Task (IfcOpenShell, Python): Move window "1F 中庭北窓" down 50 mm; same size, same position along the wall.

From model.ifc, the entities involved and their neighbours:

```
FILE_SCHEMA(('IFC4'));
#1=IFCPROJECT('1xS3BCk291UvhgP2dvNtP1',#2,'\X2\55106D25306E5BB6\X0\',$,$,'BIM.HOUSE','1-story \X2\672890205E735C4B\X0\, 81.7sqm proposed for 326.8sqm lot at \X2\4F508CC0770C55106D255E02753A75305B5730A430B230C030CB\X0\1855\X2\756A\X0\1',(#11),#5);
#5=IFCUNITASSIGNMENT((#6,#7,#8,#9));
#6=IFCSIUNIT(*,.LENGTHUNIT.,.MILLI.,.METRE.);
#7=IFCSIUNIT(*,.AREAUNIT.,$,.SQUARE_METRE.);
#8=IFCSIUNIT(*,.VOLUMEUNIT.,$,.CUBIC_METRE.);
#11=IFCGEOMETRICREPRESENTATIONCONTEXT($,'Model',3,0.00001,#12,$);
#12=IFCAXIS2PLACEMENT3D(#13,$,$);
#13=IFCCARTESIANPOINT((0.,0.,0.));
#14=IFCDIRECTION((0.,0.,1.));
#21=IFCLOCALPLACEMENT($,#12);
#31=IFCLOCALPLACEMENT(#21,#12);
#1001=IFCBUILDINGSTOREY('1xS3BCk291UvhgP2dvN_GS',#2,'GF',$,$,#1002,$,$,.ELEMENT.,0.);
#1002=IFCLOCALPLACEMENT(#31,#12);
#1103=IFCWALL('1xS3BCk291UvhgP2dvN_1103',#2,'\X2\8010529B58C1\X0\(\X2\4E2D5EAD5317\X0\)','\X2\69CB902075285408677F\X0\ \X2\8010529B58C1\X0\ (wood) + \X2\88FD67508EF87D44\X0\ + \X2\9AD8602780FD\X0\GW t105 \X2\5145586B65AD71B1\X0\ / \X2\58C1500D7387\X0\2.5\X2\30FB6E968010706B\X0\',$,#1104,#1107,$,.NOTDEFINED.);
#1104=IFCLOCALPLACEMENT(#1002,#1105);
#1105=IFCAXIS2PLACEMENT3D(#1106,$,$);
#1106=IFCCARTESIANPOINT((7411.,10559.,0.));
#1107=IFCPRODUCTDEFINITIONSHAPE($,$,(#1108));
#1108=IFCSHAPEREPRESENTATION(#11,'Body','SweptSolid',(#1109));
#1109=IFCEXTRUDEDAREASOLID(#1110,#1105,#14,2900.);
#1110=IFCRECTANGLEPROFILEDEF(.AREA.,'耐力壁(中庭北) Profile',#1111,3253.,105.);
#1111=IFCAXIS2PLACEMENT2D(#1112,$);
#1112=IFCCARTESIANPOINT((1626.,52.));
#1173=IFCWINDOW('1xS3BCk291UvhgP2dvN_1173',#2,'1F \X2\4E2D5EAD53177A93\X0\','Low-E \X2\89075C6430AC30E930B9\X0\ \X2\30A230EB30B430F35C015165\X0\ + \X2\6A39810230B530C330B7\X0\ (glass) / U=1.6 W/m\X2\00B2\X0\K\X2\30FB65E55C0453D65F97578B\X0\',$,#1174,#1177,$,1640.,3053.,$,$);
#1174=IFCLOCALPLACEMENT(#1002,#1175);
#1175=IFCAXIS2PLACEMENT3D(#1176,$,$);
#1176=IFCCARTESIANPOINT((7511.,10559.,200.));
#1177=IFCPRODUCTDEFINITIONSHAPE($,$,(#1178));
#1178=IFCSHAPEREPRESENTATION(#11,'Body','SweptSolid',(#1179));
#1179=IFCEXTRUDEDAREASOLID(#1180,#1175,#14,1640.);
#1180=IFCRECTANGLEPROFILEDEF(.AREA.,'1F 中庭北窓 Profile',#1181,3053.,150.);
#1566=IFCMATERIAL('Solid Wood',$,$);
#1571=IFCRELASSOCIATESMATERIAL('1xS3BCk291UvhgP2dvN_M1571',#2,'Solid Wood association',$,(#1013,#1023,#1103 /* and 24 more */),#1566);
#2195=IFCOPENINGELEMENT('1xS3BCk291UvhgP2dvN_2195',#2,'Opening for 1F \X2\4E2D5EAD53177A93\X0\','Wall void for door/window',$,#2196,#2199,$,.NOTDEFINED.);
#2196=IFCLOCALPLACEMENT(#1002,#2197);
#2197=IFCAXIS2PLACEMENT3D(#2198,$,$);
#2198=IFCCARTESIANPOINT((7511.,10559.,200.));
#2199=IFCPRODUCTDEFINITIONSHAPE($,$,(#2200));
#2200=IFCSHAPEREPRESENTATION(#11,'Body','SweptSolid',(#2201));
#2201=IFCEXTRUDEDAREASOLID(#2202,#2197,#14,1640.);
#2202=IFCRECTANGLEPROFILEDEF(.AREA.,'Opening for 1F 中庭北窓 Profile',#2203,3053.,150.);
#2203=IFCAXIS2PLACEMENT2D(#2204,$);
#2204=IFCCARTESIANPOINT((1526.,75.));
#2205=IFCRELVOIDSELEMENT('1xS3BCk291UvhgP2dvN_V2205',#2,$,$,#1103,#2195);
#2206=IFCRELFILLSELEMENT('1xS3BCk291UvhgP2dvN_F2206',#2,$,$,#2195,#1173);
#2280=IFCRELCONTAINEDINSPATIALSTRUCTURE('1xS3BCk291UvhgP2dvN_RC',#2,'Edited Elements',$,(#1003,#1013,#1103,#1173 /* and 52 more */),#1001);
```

```python
import numpy as np
import ifcopenshell
import ifcopenshell.api.geometry
import ifcopenshell.util.placement
import ifcopenshell.util.unit

model = ifcopenshell.open("model.ifc")
unit_scale = ifcopenshell.util.unit.calculate_unit_scale(model)

window = model.by_id(1173)
opening = window.FillsVoids[0].RelatingOpeningElement
dz = -0.05 / unit_scale

shift = np.array([0.0, 0.0, dz])
# The window is not placed relative to its opening, so move both.
for product in (opening, window):
    matrix = ifcopenshell.util.placement.get_local_placement(product.ObjectPlacement)
    matrix[:3, 3] += shift
    ifcopenshell.api.geometry.edit_object_placement(model, product=product, matrix=matrix, is_si=False)

print(f"moved by {dz * unit_scale:+.3f} m")

model.write("model_rev.ifc")
```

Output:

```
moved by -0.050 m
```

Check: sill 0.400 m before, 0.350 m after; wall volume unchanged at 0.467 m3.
